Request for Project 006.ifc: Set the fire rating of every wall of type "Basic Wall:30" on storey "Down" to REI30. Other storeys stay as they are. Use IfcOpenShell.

First a look at what the model holds.

```python
import ifcopenshell
import ifcopenshell.util.element

model = ifcopenshell.open("Project 006.ifc")
print(model.schema)
storey = next(s for s in model.by_type("IfcBuildingStorey") if s.Name == "Down")
walls = [e for e in ifcopenshell.util.element.get_decomposition(storey) if e.is_a("IfcWall")]
seen = {}
for e in walls:
    element_type = ifcopenshell.util.element.get_type(e)
    key = (element_type.Name if element_type != e and element_type else None, ifcopenshell.util.element.get_pset(e, "Pset_WallCommon", "FireRating"))
    seen[key] = seen.get(key, 0) + 1
for (name, value), count in sorted(seen.items(), key=str):
    print(count, "x", name, "|", value)
```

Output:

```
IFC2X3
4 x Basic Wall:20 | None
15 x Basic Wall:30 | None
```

```python
import ifcopenshell
import ifcopenshell.api.pset
import ifcopenshell.util.element

model = ifcopenshell.open("Project 006.ifc")

storey = next(s for s in model.by_type("IfcBuildingStorey") if s.Name == "Down")
walls = [e for e in ifcopenshell.util.element.get_decomposition(storey) if e.is_a("IfcWall")]

count = 0
for e in walls:
    element_type = ifcopenshell.util.element.get_type(e)
    if element_type in (None, e) or element_type.Name != "Basic Wall:30":
        continue
    # add_pset returns the element's existing set when there is one.
    pset = ifcopenshell.api.pset.add_pset(model, product=e, name="Pset_WallCommon")
    ifcopenshell.api.pset.edit_pset(model, pset=pset, properties={"FireRating": "REI30"})
    count += 1

print(count, "walls updated")

model.write("Project 006_v2.ifc")
```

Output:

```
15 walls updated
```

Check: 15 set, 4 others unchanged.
